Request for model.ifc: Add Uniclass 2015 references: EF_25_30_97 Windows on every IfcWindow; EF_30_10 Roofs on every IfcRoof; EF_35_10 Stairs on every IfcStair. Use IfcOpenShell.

First a look at what the model holds.

```python
import ifcopenshell

model = ifcopenshell.open("model.ifc")
print(model.schema)
print("classifications:", [c.Name for c in model.by_type("IfcClassification")])
for ifc_class in ("IfcDoor", "IfcRoof", "IfcStair", "IfcWall", "IfcWindow"):
    print(ifc_class, len(model.by_type(ifc_class)))
```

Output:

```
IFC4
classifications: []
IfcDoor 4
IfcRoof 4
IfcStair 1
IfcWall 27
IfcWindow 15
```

```python
import ifcopenshell
import ifcopenshell.api.classification

model = ifcopenshell.open("model.ifc")

system = ifcopenshell.api.classification.add_classification(model, classification="Uniclass 2015")

codes = {
    "IfcWindow": ("EF_25_30_97", "Windows"),
    "IfcRoof": ("EF_30_10", "Roofs"),
    "IfcStair": ("EF_35_10", "Stairs"),
}
for ifc_class, (code, name) in codes.items():
    products = model.by_type(ifc_class)
    ifcopenshell.api.classification.add_reference(
        model, products=products, classification=system, identification=code, name=name
    )
    print(code, len(products))

model.write("model_rev.ifc")
```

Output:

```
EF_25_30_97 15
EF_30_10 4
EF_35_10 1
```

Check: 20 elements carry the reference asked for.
